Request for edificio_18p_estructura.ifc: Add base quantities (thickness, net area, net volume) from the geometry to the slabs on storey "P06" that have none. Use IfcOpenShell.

First a look at what the model holds.

```python
import ifcopenshell
import ifcopenshell.util.element
import ifcopenshell.util.unit

model = ifcopenshell.open("edificio_18p_estructura.ifc")
print(model.schema)
for unit_type in ("LENGTHUNIT", "AREAUNIT", "VOLUMEUNIT"):
    print(unit_type, ifcopenshell.util.unit.calculate_unit_scale(model, unit_type))
storey = next(s for s in model.by_type("IfcBuildingStorey") if s.Name == "P06")
slabs = [e for e in ifcopenshell.util.element.get_decomposition(storey) if e.is_a("IfcSlab")]
for e in sorted(slabs, key=lambda e: e.id()):
    print(e.id(), e.is_a(), e.Name, list(ifcopenshell.util.element.get_psets(e, qtos_only=True)), sep=" | ")
```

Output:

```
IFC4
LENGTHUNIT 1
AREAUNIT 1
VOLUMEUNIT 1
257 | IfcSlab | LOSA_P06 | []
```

```python
import ifcopenshell
import ifcopenshell.api.pset
import ifcopenshell.geom
import ifcopenshell.util.element
import ifcopenshell.util.shape
import ifcopenshell.util.unit

model = ifcopenshell.open("edificio_18p_estructura.ifc")
unit_scale = ifcopenshell.util.unit.calculate_unit_scale(model)
area_scale = ifcopenshell.util.unit.calculate_unit_scale(model, "AREAUNIT")
volume_scale = ifcopenshell.util.unit.calculate_unit_scale(model, "VOLUMEUNIT")
settings = ifcopenshell.geom.settings()

storey = next(s for s in model.by_type("IfcBuildingStorey") if s.Name == "P06")
slabs = [e for e in ifcopenshell.util.element.get_decomposition(storey) if e.is_a("IfcSlab")]

for e in sorted(slabs, key=lambda e: e.id()):
    if ifcopenshell.util.element.get_psets(e, qtos_only=True, should_inherit=False):
        continue
    # Geometry comes back in metres, in the element's own axes.
    shape = ifcopenshell.geom.create_shape(settings, e)
    values = {
        "Width": ifcopenshell.util.shape.get_z(shape.geometry) / unit_scale,
        "NetArea": ifcopenshell.util.shape.get_footprint_area(shape.geometry) / area_scale,
        "NetVolume": ifcopenshell.util.shape.get_volume(shape.geometry) / volume_scale,
    }
    qto = ifcopenshell.api.pset.add_qto(model, product=e, name="Qto_SlabBaseQuantities")
    ifcopenshell.api.pset.edit_qto(model, qto=qto, properties=values)
    print(e.id(), {k: round(v, 3) for k, v in values.items()})

model.write("edificio_18p_estructura-out.ifc")
```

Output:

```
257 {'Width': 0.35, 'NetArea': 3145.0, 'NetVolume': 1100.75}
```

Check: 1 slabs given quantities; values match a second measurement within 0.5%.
